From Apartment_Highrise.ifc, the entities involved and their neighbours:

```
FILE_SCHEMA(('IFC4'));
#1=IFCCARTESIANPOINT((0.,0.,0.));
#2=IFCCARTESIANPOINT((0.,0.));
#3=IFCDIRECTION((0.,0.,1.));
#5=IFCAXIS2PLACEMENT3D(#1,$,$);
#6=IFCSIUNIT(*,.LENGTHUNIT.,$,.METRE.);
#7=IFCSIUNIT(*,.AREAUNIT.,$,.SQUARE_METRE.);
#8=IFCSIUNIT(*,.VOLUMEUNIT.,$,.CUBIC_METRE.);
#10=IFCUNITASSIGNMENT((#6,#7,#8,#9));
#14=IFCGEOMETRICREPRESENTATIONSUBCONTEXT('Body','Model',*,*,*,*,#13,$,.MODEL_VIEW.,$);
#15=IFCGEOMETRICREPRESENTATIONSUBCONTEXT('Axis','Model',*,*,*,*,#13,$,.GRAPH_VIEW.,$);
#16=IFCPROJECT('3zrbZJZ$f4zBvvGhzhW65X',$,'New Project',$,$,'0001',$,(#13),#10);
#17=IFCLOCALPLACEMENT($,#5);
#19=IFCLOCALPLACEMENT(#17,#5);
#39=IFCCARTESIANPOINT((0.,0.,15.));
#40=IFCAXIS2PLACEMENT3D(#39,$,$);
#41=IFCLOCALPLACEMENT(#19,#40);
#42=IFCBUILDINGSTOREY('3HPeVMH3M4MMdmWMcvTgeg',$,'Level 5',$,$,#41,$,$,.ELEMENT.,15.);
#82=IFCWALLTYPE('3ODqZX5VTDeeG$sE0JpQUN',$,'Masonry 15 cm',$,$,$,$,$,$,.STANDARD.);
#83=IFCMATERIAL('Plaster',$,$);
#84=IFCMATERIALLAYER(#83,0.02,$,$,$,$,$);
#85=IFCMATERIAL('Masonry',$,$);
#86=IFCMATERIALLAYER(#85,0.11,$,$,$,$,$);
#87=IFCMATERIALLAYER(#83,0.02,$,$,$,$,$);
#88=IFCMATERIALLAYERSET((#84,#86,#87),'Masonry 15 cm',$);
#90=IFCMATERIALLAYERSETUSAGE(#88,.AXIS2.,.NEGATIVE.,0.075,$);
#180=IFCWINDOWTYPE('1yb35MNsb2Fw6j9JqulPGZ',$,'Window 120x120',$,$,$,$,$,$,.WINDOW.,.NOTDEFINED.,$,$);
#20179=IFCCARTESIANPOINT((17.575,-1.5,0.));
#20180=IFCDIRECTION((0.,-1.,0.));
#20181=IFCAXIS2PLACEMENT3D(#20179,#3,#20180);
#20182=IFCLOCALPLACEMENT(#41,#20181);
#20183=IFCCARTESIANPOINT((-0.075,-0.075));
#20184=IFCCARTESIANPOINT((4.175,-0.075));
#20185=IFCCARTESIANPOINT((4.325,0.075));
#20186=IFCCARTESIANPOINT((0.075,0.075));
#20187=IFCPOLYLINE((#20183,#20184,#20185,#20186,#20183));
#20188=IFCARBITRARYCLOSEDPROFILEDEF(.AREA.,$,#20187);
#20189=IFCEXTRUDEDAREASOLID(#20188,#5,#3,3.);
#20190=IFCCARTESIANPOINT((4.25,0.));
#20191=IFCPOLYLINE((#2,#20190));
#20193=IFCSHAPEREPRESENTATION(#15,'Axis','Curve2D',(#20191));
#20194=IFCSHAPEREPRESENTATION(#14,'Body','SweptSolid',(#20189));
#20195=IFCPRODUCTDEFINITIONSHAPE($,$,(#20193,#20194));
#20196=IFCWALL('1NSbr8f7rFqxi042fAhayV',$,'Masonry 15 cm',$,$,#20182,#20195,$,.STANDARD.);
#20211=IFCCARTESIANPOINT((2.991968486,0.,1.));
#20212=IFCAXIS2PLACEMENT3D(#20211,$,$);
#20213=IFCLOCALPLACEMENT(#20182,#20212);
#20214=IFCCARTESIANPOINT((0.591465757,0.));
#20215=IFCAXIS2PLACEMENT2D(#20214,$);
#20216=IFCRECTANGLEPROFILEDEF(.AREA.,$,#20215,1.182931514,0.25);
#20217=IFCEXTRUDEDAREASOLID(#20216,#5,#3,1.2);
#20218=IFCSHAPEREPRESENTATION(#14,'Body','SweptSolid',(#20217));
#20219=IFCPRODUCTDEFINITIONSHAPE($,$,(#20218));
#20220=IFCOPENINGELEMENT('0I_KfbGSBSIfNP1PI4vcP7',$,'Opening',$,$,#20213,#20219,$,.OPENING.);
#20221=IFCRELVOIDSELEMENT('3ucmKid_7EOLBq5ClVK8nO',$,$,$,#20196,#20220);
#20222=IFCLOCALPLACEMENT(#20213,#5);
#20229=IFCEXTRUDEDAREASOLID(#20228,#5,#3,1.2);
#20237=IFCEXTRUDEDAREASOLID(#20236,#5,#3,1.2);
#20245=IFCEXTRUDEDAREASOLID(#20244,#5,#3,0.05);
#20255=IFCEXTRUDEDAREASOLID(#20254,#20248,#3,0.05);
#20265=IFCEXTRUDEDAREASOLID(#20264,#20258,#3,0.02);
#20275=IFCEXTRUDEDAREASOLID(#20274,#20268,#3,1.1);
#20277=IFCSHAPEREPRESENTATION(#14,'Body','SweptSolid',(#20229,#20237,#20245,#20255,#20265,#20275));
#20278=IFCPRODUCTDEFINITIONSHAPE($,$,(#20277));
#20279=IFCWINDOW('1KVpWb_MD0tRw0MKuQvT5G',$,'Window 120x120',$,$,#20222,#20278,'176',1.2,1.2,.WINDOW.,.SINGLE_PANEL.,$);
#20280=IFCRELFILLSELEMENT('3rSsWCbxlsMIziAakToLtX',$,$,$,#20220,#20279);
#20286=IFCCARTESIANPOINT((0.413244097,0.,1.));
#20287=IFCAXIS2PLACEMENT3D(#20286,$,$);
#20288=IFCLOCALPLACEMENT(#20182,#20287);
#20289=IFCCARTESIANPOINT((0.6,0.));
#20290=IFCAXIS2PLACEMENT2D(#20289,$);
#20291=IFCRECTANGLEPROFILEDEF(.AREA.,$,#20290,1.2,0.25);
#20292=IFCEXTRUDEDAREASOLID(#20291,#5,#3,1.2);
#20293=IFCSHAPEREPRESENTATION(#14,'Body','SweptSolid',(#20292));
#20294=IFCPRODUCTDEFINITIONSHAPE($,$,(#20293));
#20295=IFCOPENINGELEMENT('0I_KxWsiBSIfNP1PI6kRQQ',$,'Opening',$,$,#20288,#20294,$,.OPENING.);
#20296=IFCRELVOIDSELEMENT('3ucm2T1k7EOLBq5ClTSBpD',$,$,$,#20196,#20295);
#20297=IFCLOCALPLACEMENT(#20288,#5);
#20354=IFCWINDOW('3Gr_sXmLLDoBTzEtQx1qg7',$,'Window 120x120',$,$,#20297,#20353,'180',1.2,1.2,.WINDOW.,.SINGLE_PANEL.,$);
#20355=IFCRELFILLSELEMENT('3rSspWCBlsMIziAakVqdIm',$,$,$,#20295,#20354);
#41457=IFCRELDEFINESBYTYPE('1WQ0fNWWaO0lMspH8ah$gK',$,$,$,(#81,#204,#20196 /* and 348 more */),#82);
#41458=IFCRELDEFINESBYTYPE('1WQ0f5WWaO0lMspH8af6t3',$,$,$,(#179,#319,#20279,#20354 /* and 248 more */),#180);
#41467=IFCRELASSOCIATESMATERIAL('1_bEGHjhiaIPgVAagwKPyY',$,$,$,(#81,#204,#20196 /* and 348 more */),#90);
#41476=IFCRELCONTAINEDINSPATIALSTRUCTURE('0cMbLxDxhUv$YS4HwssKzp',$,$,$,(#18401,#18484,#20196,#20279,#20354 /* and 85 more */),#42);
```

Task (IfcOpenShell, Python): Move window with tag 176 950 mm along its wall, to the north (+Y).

```python
import ifcopenshell
import ifcopenshell.api.geometry
import ifcopenshell.util.placement
import ifcopenshell.util.unit

model = ifcopenshell.open("Apartment_Highrise.ifc")
unit_scale = ifcopenshell.util.unit.calculate_unit_scale(model)

window = model.by_guid("1KVpWb_MD0tRw0MKuQvT5G")
opening = window.FillsVoids[0].RelatingOpeningElement
wall = opening.VoidsElements[0].RelatingBuildingElement

wall_matrix = ifcopenshell.util.placement.get_local_placement(wall.ObjectPlacement)
shift = wall_matrix[:3, 0] * -0.95 / unit_scale
before = ifcopenshell.util.placement.get_local_placement(window.ObjectPlacement)[:3, 3].copy()

# The window is placed relative to its opening, so it follows when the opening moves.
matrix = ifcopenshell.util.placement.get_local_placement(opening.ObjectPlacement)
matrix[:3, 3] += shift
ifcopenshell.api.geometry.edit_object_placement(
    model, product=opening, matrix=matrix, is_si=False, should_transform_children=True
)

after = ifcopenshell.util.placement.get_local_placement(window.ObjectPlacement)[:3, 3]
print("window moved by", (after - before).round(3) + 0.0)

model.write("Apartment_Highrise_edited.ifc")
```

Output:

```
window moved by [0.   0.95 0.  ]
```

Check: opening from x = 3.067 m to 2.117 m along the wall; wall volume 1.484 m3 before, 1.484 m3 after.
